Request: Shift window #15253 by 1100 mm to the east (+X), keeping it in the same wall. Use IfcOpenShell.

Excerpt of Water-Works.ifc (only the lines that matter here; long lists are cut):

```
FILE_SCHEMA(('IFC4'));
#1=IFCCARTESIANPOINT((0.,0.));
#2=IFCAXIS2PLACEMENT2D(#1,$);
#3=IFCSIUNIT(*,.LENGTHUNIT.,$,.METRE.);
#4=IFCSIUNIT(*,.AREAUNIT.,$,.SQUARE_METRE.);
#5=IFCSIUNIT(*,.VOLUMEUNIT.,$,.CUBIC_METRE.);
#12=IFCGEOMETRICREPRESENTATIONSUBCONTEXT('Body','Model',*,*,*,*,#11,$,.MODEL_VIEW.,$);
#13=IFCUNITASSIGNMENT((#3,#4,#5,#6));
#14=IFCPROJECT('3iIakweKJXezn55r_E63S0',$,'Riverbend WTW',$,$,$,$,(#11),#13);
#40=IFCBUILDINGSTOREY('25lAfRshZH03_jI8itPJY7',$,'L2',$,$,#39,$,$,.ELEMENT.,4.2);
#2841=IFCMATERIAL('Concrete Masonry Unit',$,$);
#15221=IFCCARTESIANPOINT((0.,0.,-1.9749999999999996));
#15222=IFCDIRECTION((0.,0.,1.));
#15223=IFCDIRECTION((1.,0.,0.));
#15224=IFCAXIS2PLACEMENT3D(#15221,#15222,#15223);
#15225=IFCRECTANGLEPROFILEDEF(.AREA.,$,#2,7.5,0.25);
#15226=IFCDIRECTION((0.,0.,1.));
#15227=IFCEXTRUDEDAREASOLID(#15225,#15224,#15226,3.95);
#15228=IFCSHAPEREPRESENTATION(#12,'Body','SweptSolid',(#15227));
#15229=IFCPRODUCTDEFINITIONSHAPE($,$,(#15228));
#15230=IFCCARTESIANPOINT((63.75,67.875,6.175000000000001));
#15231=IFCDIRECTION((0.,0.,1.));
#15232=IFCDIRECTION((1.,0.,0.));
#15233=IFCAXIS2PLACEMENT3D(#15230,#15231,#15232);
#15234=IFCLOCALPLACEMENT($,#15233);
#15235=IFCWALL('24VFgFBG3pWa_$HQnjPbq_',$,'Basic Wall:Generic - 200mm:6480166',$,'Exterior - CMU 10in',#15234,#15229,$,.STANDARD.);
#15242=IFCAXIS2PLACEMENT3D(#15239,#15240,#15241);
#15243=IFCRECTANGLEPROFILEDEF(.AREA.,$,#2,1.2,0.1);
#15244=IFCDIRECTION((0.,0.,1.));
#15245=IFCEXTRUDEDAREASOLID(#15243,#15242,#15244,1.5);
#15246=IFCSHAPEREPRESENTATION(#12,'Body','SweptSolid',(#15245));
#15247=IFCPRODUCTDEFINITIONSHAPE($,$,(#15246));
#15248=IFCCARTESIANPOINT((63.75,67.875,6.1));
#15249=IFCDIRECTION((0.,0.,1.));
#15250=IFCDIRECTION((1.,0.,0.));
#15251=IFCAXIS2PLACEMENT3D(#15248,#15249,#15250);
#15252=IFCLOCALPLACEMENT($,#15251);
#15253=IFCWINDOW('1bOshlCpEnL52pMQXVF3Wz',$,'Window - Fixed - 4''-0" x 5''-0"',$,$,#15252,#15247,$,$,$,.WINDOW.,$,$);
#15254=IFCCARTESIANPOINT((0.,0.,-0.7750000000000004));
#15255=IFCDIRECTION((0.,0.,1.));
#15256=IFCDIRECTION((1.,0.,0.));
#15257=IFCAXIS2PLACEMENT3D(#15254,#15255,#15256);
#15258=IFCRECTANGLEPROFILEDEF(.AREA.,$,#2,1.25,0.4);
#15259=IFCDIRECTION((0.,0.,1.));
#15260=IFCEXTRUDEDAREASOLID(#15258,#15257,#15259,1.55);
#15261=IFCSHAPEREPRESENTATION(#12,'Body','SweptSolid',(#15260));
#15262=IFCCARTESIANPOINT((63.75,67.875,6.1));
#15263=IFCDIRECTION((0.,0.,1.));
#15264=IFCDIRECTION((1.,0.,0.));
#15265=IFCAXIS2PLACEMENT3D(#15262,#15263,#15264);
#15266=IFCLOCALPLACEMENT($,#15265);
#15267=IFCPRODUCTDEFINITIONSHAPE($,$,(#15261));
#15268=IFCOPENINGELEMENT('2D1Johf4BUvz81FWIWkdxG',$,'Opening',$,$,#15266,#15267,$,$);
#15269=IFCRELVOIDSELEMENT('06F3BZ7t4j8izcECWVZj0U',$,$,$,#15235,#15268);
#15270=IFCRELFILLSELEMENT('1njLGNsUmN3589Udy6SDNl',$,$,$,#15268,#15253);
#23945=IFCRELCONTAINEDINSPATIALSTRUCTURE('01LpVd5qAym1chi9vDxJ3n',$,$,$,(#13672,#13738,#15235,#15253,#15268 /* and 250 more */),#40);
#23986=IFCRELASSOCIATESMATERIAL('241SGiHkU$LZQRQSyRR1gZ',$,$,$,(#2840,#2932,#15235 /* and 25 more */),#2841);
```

```python
import ifcopenshell
import ifcopenshell.api.geometry
import ifcopenshell.util.placement
import ifcopenshell.util.unit

model = ifcopenshell.open("Water-Works.ifc")
unit_scale = ifcopenshell.util.unit.calculate_unit_scale(model)

window = model.by_guid("1bOshlCpEnL52pMQXVF3Wz")
opening = window.FillsVoids[0].RelatingOpeningElement
wall = opening.VoidsElements[0].RelatingBuildingElement

wall_matrix = ifcopenshell.util.placement.get_local_placement(wall.ObjectPlacement)
shift = wall_matrix[:3, 0] * 1.1 / unit_scale
before = ifcopenshell.util.placement.get_local_placement(window.ObjectPlacement)[:3, 3].copy()

# The window is not placed relative to its opening, so move both.
for product in (opening, window):
    matrix = ifcopenshell.util.placement.get_local_placement(product.ObjectPlacement)
    matrix[:3, 3] += shift
    ifcopenshell.api.geometry.edit_object_placement(model, product=product, matrix=matrix, is_si=False)

after = ifcopenshell.util.placement.get_local_placement(window.ObjectPlacement)[:3, 3]
print("window moved by", (after - before).round(3) + 0.0)

model.write("Water-Works_rev.ifc")
```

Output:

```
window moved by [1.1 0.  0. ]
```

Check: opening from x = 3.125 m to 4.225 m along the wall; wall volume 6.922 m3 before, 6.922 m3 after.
